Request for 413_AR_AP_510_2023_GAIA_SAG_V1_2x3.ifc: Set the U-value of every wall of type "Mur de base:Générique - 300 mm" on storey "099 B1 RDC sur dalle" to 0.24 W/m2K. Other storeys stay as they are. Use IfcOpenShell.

First a look at what the model holds.

```python
import ifcopenshell
import ifcopenshell.util.element

model = ifcopenshell.open("413_AR_AP_510_2023_GAIA_SAG_V1_2x3.ifc")
print(model.schema)
storey = next(s for s in model.by_type("IfcBuildingStorey") if s.Name == "099 B1 RDC sur dalle")
walls = [e for e in ifcopenshell.util.element.get_decomposition(storey) if e.is_a("IfcWall")]
seen = {}
for e in walls:
    element_type = ifcopenshell.util.element.get_type(e)
    key = (element_type.Name if element_type != e and element_type else None, ifcopenshell.util.element.get_pset(e, "Pset_WallCommon", "ThermalTransmittance"))
    seen[key] = seen.get(key, 0) + 1
for (name, value), count in sorted(seen.items(), key=str):
    print(count, "x", name, "|", value)
```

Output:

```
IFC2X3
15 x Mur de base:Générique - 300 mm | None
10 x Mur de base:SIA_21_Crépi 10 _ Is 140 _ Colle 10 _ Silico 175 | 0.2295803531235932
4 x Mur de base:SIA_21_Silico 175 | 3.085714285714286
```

```python
import ifcopenshell
import ifcopenshell.api.pset
import ifcopenshell.util.element

model = ifcopenshell.open("413_AR_AP_510_2023_GAIA_SAG_V1_2x3.ifc")

storey = next(s for s in model.by_type("IfcBuildingStorey") if s.Name == "099 B1 RDC sur dalle")
walls = [e for e in ifcopenshell.util.element.get_decomposition(storey) if e.is_a("IfcWall")]

count = 0
for e in walls:
    element_type = ifcopenshell.util.element.get_type(e)
    if element_type in (None, e) or element_type.Name != "Mur de base:Générique - 300 mm":
        continue
    # add_pset returns the element's existing set when there is one.
    pset = ifcopenshell.api.pset.add_pset(model, product=e, name="Pset_WallCommon")
    ifcopenshell.api.pset.edit_pset(model, pset=pset, properties={"ThermalTransmittance": 0.24})
    count += 1

print(count, "walls updated")

model.write("413_AR_AP_510_2023_GAIA_SAG_V1_2x3_edited.ifc")
```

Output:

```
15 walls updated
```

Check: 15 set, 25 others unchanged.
